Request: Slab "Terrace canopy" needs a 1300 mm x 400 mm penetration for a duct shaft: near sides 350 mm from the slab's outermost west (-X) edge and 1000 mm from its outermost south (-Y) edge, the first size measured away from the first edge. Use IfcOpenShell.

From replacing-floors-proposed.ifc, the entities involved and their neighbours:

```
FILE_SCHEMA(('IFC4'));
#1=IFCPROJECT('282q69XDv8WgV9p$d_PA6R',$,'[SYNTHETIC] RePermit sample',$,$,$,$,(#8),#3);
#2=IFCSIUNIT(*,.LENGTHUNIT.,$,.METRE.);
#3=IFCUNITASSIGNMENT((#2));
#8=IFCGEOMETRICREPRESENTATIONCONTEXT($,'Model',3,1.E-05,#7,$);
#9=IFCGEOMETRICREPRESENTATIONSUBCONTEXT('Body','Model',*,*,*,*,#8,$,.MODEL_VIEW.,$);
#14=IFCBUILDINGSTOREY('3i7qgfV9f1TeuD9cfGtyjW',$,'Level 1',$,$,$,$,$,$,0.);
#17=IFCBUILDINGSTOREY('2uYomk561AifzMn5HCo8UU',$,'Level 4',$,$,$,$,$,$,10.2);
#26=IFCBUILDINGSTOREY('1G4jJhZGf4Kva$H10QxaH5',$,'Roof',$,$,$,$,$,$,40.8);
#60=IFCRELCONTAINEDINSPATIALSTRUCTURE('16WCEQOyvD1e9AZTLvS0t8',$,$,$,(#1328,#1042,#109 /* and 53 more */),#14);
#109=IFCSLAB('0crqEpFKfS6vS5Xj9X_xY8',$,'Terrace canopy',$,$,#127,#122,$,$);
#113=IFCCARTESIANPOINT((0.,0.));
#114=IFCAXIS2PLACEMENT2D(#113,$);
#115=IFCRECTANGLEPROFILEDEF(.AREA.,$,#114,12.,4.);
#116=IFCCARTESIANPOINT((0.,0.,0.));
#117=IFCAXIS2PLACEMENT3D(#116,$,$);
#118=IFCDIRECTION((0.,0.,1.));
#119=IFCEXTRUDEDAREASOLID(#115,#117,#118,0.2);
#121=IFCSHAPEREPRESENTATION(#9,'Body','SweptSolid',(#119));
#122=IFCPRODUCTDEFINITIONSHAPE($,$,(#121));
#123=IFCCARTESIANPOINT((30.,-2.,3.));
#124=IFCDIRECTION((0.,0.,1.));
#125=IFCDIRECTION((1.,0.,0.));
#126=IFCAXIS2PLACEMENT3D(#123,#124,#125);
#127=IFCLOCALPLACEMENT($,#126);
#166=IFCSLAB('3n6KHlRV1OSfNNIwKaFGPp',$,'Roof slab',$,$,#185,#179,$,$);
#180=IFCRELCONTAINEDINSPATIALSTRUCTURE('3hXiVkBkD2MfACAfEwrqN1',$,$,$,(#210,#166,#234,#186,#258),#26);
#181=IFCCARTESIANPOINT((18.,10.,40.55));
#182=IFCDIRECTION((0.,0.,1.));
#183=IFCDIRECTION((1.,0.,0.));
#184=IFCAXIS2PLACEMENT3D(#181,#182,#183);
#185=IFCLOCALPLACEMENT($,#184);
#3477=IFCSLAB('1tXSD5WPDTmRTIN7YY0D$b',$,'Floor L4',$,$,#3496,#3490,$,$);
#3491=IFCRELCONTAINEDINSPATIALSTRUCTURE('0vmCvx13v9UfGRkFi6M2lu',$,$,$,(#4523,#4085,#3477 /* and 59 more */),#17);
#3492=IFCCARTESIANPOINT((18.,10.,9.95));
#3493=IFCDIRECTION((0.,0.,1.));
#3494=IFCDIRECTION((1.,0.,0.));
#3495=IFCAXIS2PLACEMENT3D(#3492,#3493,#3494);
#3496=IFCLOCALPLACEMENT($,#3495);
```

```python
import numpy as np
import ifcopenshell
import ifcopenshell.api.feature
import ifcopenshell.api.geometry
import ifcopenshell.api.root
import ifcopenshell.geom
import ifcopenshell.util.placement
import ifcopenshell.util.representation
import ifcopenshell.util.shape
import ifcopenshell.util.unit

model = ifcopenshell.open("replacing-floors-proposed.ifc")
unit_scale = ifcopenshell.util.unit.calculate_unit_scale(model)
settings = ifcopenshell.geom.settings()


def volume(element):
    """Net volume in cubic metres, openings subtracted."""
    shape = ifcopenshell.geom.create_shape(settings, element)
    return ifcopenshell.util.shape.get_volume(shape.geometry)


slab = model.by_id(109)
before = volume(slab)

# Extent in the slab's own axes, in metres. The edges named are its -X and -Y sides.
slab_shape = ifcopenshell.geom.create_shape(settings, slab)
vertices = ifcopenshell.util.shape.get_vertices(slab_shape.geometry)
x_min, y_min, bottom = vertices.min(axis=0)
top = vertices[:, 2].max()

opening = ifcopenshell.api.root.create_entity(model, ifc_class="IfcOpeningElement", name="Duct shaft opening", predefined_type="OPENING")
context = ifcopenshell.util.representation.get_context(model, "Model", "Body", "MODEL_VIEW")
width, depth = 1.3, 0.4
outline = [(0.0, 0.0), (width, 0.0), (width, depth), (0.0, depth), (0.0, 0.0)]
# Overshoot both faces by 50 mm so the cut is clean.
shape = ifcopenshell.api.geometry.add_slab_representation(
    model, context=context, depth=top - bottom + 0.1, polyline=outline
)
ifcopenshell.api.geometry.assign_representation(model, product=opening, representation=shape)

matrix = ifcopenshell.util.placement.get_local_placement(slab.ObjectPlacement)
matrix[:, 3] = matrix @ np.append(np.array([x_min + 0.35, y_min + 1, bottom - 0.05]) / unit_scale, 1.0)
ifcopenshell.api.geometry.edit_object_placement(model, product=opening, matrix=matrix, is_si=False)
ifcopenshell.api.feature.add_feature(model, feature=opening, element=slab)

after = volume(slab)

print(f"slab volume {before:.3f} -> {after:.3f} m3")

model.write("replacing-floors-proposed_v2.ifc")
```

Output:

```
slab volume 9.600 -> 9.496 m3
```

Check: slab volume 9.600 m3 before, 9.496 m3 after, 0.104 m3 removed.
